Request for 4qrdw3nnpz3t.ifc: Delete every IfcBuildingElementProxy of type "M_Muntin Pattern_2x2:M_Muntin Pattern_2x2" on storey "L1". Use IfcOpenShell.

First a look at what the model holds.

```python
import ifcopenshell
import ifcopenshell.util.element

model = ifcopenshell.open("4qrdw3nnpz3t.ifc")
print(model.schema)
storey = next(s for s in model.by_type("IfcBuildingStorey") if s.Name == "L1")
proxies = [e for e in ifcopenshell.util.element.get_decomposition(storey) if e.is_a("IfcBuildingElementProxy")]
seen = {}
for e in proxies:
    element_type = ifcopenshell.util.element.get_type(e)
    name = element_type.Name if element_type not in (None, e) else None
    seen[name] = seen.get(name, 0) + 1
for name, count in sorted(seen.items(), key=str):
    print(count, "x", name)
```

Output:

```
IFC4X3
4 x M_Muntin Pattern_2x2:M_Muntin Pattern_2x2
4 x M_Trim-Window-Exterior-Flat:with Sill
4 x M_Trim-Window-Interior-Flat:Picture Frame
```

```python
import ifcopenshell
import ifcopenshell.api.root
import ifcopenshell.util.element

model = ifcopenshell.open("4qrdw3nnpz3t.ifc")

storey = next(s for s in model.by_type("IfcBuildingStorey") if s.Name == "L1")
proxies = [e for e in ifcopenshell.util.element.get_decomposition(storey) if e.is_a("IfcBuildingElementProxy")]
targets = [e for e in proxies if (t := ifcopenshell.util.element.get_type(e)) not in (None, e) and t.Name == "M_Muntin Pattern_2x2:M_Muntin Pattern_2x2"]

for e in targets:
    ifcopenshell.api.root.remove_product(model, product=e)
print(len(targets), "removed")

model.write("4qrdw3nnpz3t_updated.ifc")
```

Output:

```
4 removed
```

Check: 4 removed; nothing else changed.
